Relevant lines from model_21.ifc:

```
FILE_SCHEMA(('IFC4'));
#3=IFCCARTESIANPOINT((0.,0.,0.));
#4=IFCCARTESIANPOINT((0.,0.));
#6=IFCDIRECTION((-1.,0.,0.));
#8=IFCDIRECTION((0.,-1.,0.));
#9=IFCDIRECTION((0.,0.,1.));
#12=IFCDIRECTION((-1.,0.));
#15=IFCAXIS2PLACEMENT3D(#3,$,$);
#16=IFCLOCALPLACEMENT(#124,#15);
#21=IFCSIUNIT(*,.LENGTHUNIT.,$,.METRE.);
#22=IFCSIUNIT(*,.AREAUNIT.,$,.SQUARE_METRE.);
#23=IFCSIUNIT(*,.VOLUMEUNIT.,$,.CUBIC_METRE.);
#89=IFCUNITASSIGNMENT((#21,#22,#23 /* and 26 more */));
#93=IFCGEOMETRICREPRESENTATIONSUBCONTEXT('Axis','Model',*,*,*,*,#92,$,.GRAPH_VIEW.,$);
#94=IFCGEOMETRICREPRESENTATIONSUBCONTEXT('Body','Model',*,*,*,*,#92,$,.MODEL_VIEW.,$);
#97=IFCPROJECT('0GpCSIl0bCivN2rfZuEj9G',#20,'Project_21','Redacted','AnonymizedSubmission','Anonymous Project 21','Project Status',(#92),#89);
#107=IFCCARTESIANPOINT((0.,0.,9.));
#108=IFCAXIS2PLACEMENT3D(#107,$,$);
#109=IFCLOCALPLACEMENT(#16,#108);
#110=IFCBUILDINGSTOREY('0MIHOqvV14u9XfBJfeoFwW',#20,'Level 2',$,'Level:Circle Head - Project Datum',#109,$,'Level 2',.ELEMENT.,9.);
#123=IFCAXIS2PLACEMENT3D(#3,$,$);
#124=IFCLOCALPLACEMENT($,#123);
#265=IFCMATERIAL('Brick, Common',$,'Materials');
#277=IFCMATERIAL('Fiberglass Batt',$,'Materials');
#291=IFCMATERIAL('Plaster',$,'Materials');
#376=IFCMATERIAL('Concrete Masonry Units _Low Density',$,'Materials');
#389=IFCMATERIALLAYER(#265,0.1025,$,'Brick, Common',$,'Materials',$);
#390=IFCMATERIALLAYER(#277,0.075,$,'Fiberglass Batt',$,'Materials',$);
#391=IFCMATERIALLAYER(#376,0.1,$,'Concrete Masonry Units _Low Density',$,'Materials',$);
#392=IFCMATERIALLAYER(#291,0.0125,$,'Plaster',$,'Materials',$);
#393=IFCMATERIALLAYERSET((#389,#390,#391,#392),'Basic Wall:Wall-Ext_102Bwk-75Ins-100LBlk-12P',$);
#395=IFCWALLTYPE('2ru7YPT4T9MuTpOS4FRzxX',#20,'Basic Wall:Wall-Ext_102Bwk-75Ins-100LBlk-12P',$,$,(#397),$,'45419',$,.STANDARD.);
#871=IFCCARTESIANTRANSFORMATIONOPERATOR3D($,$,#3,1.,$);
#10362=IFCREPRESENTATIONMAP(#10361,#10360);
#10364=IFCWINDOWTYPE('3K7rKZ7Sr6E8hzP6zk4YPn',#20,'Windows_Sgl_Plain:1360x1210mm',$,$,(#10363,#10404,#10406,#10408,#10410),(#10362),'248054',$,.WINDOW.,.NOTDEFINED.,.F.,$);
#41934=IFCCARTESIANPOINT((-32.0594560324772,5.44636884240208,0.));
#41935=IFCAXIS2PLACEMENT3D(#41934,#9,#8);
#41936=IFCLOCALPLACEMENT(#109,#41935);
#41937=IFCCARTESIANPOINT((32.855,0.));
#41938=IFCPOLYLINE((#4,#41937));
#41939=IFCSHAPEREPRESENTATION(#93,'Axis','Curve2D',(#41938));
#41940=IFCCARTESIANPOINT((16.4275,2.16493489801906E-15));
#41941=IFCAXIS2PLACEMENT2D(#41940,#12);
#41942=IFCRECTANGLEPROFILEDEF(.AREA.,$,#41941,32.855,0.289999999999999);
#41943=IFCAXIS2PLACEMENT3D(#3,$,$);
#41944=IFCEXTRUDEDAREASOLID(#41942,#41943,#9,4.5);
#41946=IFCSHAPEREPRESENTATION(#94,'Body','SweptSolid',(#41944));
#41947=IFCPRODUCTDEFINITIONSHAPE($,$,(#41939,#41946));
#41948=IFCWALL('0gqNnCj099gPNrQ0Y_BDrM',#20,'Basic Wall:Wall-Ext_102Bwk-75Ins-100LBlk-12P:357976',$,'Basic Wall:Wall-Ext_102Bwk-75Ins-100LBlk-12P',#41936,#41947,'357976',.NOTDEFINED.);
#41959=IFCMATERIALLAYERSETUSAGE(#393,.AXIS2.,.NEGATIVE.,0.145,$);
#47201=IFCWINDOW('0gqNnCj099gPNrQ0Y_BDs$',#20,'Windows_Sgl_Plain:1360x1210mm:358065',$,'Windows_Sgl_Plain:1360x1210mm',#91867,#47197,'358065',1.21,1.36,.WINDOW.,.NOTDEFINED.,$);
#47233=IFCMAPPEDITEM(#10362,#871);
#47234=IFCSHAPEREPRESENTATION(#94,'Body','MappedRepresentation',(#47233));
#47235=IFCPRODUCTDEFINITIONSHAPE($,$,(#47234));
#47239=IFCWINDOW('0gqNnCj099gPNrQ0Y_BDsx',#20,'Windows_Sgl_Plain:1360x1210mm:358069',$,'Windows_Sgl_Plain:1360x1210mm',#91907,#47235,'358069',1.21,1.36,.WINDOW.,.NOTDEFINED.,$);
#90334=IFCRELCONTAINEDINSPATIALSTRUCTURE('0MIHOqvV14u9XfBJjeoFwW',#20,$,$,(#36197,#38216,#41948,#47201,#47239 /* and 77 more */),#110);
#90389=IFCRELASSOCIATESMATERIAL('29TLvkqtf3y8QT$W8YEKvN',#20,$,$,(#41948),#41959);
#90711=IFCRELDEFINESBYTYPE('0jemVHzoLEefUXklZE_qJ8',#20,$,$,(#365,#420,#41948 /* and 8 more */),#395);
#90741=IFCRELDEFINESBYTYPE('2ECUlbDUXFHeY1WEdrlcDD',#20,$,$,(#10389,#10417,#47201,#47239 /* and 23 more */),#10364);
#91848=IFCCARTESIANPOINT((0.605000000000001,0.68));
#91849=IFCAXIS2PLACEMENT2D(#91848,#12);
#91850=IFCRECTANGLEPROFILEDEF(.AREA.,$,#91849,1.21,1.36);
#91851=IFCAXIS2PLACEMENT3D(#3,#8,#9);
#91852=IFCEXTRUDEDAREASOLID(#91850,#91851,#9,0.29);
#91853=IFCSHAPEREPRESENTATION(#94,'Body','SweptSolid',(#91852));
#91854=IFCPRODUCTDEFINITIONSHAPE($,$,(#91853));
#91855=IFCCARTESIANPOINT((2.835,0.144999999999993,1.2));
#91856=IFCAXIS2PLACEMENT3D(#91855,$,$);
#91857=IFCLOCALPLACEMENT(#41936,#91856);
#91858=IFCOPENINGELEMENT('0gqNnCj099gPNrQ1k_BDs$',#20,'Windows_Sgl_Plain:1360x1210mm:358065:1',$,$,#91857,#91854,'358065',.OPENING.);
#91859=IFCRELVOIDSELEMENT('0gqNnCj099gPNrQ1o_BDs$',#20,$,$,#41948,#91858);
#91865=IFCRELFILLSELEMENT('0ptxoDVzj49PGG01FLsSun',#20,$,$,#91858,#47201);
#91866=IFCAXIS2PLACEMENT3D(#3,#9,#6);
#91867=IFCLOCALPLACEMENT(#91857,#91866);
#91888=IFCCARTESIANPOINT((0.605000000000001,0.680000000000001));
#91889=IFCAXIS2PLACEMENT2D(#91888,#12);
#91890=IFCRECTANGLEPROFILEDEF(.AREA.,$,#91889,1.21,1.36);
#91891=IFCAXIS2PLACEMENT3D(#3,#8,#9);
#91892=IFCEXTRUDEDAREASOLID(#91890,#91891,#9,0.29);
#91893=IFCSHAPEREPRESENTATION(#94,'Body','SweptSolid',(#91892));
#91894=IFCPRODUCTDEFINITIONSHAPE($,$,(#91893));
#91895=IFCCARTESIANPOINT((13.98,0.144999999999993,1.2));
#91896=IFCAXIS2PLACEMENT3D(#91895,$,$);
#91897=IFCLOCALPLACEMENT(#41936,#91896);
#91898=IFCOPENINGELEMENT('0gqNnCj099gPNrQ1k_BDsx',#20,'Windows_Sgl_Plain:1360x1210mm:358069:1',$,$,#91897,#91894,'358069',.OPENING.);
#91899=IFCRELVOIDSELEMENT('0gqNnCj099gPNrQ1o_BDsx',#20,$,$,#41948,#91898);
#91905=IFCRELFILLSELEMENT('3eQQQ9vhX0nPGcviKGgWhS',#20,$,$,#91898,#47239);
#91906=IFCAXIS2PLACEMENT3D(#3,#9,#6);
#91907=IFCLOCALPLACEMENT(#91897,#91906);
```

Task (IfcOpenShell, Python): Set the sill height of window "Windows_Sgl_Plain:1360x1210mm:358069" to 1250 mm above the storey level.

```python
import numpy as np
import ifcopenshell
import ifcopenshell.api.geometry
import ifcopenshell.geom
import ifcopenshell.util.element
import ifcopenshell.util.placement
import ifcopenshell.util.shape
import ifcopenshell.util.unit

model = ifcopenshell.open("model_21.ifc")
unit_scale = ifcopenshell.util.unit.calculate_unit_scale(model)

window = model.by_guid("0gqNnCj099gPNrQ0Y_BDsx")
opening = window.FillsVoids[0].RelatingOpeningElement
storey = ifcopenshell.util.element.get_container(window, ifc_class="IfcBuildingStorey")
level = ifcopenshell.util.placement.get_local_placement(storey.ObjectPlacement)[2, 3]

# The opening's origin need not be at the sill, so measure its lowest point.
shape = ifcopenshell.geom.create_shape(ifcopenshell.geom.settings(), opening)
bottom = ifcopenshell.util.shape.get_shape_bottom_elevation(shape, shape.geometry) / unit_scale
dz = level + 1.25 / unit_scale - bottom

shift = np.array([0.0, 0.0, dz])
# The window is placed relative to its opening, so it follows when the opening moves.
matrix = ifcopenshell.util.placement.get_local_placement(opening.ObjectPlacement)
matrix[:3, 3] += shift
ifcopenshell.api.geometry.edit_object_placement(
    model, product=opening, matrix=matrix, is_si=False, should_transform_children=True
)

print(f"moved by {dz * unit_scale:+.3f} m")

model.write("model_21_rev.ifc")
```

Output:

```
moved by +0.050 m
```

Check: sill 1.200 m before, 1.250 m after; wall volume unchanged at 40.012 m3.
